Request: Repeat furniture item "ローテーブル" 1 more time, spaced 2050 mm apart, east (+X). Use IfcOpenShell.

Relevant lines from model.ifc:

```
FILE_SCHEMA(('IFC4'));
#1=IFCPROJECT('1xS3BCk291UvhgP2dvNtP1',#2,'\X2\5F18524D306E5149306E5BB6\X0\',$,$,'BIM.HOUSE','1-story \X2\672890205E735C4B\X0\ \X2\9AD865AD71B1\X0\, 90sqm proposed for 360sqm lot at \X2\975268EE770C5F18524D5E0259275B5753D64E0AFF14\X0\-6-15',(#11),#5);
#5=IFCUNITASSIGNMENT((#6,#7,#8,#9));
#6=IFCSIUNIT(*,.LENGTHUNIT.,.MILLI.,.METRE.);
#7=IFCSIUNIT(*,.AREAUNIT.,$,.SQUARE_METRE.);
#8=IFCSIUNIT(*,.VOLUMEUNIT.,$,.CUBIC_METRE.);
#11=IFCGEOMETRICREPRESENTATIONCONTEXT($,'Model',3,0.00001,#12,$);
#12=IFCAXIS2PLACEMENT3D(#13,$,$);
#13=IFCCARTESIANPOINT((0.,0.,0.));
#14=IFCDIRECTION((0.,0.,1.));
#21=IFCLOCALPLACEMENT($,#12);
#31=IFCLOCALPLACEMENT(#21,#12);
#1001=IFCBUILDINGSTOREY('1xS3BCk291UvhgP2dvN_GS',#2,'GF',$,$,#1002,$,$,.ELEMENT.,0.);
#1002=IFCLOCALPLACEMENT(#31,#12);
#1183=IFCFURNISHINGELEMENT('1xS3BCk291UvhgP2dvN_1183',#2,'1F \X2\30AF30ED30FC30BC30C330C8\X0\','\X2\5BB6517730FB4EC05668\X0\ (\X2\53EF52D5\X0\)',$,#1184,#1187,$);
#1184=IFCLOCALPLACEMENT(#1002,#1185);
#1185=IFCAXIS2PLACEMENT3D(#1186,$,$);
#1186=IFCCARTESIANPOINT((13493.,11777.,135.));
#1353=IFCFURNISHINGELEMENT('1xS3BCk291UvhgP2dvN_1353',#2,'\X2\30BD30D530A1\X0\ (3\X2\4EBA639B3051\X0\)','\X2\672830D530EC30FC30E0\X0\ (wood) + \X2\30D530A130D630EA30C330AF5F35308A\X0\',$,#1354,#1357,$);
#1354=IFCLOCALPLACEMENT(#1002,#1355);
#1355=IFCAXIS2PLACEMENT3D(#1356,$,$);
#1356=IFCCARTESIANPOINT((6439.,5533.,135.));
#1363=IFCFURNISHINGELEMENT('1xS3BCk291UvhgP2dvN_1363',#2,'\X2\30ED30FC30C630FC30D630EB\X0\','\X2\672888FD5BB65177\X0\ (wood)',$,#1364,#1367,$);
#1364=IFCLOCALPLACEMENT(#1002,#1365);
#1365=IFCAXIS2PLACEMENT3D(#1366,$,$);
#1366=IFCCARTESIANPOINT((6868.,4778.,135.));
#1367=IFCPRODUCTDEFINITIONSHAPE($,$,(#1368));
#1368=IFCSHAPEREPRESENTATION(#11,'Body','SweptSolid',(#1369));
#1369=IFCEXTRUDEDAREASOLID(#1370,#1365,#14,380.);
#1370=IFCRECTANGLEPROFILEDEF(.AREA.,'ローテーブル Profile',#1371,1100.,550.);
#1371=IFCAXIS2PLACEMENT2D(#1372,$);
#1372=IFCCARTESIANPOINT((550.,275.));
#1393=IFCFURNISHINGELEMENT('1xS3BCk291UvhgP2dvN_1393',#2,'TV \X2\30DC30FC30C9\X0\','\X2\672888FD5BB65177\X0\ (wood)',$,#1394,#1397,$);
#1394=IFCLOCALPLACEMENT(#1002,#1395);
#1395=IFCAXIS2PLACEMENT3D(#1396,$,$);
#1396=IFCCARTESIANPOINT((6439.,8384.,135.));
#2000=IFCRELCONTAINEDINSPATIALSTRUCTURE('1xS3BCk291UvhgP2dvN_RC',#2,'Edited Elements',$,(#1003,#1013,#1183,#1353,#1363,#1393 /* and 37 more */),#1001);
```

```python
import numpy as np
import ifcopenshell
import ifcopenshell.api.geometry
import ifcopenshell.api.root
import ifcopenshell.util.element
import ifcopenshell.util.placement
import ifcopenshell.util.unit

model = ifcopenshell.open("model.ifc")
unit_scale = ifcopenshell.util.unit.calculate_unit_scale(model)


def reuse_history(source, copy):
    """copy_class also copies each property set's owner history, people and application; keep the originals."""
    for rel in copy.IsDefinedBy:
        if rel.is_a("IfcRelDefinesByProperties") and (history := rel.RelatingPropertyDefinition.OwnerHistory):
            rel.RelatingPropertyDefinition.OwnerHistory = source.OwnerHistory
            ifcopenshell.util.element.remove_deep2(model, history)


source = model.by_guid("1xS3BCk291UvhgP2dvN_1363")
base = ifcopenshell.util.placement.get_local_placement(source.ObjectPlacement)
step = np.array([1.0, 0.0, 0.0]) * 2.05 / unit_scale

for i in range(1, 2):
    copy = ifcopenshell.api.root.copy_class(model, product=source)
    copy.Representation = ifcopenshell.util.element.copy_deep(
        model, source.Representation, exclude=["IfcGeometricRepresentationContext", "IfcRepresentationMap"]
    )
    reuse_history(source, copy)
    matrix = base.copy()
    matrix[:3, 3] += i * step
    print("added at", matrix[:3, 3].round(3) + 0.0)
    ifcopenshell.api.geometry.edit_object_placement(model, product=copy, matrix=matrix, is_si=False)

model.write("model-out.ifc")
```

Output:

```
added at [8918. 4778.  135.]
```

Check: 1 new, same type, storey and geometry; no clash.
